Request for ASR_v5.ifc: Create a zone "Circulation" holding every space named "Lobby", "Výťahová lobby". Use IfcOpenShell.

First a look at what the model holds.

```python
import ifcopenshell

model = ifcopenshell.open("ASR_v5.ifc")
print(model.schema)
seen = {}
for space in model.by_type("IfcSpace"):
    seen[space.LongName] = seen.get(space.LongName, 0) + 1
for name, count in sorted(seen.items(), key=str):
    print(count, "x", name)
print("zones:", [z.Name for z in model.by_type("IfcZone")][:20])
```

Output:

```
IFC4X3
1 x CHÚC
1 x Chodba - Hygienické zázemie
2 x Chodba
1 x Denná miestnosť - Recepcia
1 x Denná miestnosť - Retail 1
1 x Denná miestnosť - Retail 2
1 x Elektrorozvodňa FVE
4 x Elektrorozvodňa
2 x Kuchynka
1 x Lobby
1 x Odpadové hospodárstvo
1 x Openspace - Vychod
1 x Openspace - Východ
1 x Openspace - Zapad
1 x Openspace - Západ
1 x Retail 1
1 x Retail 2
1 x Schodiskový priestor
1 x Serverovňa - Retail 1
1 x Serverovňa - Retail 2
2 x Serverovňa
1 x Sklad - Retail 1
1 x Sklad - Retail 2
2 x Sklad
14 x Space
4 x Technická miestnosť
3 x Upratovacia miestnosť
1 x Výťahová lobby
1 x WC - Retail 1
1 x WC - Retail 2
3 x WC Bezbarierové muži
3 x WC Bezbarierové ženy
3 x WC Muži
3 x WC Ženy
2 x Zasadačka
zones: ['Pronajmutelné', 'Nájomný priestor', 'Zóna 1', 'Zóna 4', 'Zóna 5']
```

```python
import ifcopenshell
import ifcopenshell.api.group
import ifcopenshell.api.root

model = ifcopenshell.open("ASR_v5.ifc")

names = {"Lobby", "Výťahová lobby"}
spaces = [s for s in model.by_type("IfcSpace") if s.LongName in names]

zone = ifcopenshell.api.root.create_entity(model, ifc_class="IfcZone", name="Circulation")
ifcopenshell.api.group.assign_group(model, products=spaces, group=zone)
print(len(spaces), "spaces in", zone.Name)

model.write("ASR_v5_v2.ifc")
```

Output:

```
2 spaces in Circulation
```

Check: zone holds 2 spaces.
